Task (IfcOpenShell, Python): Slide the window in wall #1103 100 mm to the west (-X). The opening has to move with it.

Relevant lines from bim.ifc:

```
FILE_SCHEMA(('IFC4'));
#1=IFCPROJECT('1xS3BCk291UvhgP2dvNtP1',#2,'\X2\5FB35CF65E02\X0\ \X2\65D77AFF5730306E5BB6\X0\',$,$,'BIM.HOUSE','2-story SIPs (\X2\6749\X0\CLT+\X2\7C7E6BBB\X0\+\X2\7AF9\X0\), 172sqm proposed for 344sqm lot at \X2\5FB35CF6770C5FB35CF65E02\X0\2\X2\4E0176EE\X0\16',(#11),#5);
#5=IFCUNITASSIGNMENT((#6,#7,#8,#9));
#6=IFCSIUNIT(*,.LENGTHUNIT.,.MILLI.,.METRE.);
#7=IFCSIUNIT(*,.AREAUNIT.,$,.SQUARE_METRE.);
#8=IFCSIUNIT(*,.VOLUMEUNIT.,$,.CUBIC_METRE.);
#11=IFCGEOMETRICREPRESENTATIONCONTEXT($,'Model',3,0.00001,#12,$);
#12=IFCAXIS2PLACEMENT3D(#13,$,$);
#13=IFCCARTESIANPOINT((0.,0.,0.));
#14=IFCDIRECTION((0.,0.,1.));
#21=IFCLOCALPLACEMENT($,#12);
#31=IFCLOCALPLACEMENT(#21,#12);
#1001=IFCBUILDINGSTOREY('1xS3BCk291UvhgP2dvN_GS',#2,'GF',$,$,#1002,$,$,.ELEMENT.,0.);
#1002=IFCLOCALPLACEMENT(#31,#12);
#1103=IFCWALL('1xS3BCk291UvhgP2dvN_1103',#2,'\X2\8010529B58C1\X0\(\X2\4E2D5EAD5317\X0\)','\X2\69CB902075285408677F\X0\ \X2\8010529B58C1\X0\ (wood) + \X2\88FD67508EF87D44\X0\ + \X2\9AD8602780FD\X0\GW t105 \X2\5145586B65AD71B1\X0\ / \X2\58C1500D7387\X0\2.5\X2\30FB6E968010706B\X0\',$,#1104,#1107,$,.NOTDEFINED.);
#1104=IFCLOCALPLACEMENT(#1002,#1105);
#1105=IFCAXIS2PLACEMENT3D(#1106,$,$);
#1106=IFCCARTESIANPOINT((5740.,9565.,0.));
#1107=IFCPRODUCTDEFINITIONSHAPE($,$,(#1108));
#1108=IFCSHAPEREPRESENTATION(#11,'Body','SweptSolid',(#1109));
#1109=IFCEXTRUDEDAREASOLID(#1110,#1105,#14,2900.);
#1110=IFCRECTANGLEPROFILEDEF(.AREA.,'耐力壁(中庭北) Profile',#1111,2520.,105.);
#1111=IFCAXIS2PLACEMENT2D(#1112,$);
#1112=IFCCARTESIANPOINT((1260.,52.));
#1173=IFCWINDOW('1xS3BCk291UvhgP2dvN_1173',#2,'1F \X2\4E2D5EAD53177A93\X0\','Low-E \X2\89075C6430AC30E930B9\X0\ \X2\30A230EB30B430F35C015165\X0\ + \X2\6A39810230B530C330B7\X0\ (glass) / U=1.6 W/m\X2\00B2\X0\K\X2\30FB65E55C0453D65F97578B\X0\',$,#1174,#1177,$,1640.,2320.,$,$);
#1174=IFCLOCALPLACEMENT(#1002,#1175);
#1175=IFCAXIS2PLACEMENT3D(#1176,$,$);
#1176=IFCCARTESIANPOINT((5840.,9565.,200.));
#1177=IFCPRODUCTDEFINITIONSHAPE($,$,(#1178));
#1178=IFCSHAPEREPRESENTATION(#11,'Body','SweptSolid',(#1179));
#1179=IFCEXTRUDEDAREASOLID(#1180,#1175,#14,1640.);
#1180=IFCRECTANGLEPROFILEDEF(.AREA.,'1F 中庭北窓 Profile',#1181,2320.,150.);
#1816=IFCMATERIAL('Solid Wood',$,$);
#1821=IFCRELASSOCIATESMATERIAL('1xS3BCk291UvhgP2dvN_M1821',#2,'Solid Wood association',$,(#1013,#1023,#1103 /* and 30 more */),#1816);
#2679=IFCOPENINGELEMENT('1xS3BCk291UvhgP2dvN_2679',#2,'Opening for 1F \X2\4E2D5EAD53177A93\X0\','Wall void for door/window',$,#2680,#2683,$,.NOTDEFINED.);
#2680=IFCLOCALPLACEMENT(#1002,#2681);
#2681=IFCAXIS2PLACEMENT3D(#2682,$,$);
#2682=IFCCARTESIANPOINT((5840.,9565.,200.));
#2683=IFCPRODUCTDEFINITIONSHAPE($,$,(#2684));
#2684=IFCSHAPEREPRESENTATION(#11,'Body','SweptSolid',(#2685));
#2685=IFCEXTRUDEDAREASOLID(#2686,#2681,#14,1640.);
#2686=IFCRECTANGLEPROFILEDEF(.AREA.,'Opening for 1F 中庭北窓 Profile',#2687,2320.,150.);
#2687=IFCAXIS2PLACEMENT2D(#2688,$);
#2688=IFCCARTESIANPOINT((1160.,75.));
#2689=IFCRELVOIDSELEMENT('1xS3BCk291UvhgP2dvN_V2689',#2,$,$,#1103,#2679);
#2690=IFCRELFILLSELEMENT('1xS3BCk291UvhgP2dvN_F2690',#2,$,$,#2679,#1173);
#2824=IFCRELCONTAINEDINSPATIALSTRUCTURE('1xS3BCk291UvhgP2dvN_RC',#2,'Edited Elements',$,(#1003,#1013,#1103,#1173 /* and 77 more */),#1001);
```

```python
import ifcopenshell
import ifcopenshell.api.geometry
import ifcopenshell.util.placement
import ifcopenshell.util.unit

model = ifcopenshell.open("bim.ifc")
unit_scale = ifcopenshell.util.unit.calculate_unit_scale(model)

window = model.by_id(1173)
opening = window.FillsVoids[0].RelatingOpeningElement
wall = opening.VoidsElements[0].RelatingBuildingElement

wall_matrix = ifcopenshell.util.placement.get_local_placement(wall.ObjectPlacement)
shift = wall_matrix[:3, 0] * -0.1 / unit_scale
before = ifcopenshell.util.placement.get_local_placement(window.ObjectPlacement)[:3, 3].copy()

# The window is not placed relative to its opening, so move both.
for product in (opening, window):
    matrix = ifcopenshell.util.placement.get_local_placement(product.ObjectPlacement)
    matrix[:3, 3] += shift
    ifcopenshell.api.geometry.edit_object_placement(model, product=product, matrix=matrix, is_si=False)

after = ifcopenshell.util.placement.get_local_placement(window.ObjectPlacement)[:3, 3]
print("window moved by", (after - before).round(3) + 0.0)

model.write("bim-out.ifc")
```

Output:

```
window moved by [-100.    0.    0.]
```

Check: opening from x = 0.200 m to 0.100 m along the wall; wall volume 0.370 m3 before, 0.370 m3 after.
